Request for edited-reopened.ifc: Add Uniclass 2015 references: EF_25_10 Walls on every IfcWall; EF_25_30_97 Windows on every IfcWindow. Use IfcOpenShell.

First a look at what the model holds.

```python
import ifcopenshell

model = ifcopenshell.open("edited-reopened.ifc")
print(model.schema)
print("classifications:", [c.Name for c in model.by_type("IfcClassification")])
for ifc_class in ("IfcDoor", "IfcRoof", "IfcStair", "IfcWall", "IfcWindow"):
    print(ifc_class, len(model.by_type(ifc_class)))
```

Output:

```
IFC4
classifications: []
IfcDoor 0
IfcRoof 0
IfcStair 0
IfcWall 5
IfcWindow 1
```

```python
import ifcopenshell
import ifcopenshell.api.classification

model = ifcopenshell.open("edited-reopened.ifc")

system = ifcopenshell.api.classification.add_classification(model, classification="Uniclass 2015")

codes = {
    "IfcWall": ("EF_25_10", "Walls"),
    "IfcWindow": ("EF_25_30_97", "Windows"),
}
for ifc_class, (code, name) in codes.items():
    products = model.by_type(ifc_class)
    ifcopenshell.api.classification.add_reference(
        model, products=products, classification=system, identification=code, name=name
    )
    print(code, len(products))

model.write("edited-reopened_updated.ifc")
```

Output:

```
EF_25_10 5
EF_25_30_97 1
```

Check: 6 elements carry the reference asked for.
